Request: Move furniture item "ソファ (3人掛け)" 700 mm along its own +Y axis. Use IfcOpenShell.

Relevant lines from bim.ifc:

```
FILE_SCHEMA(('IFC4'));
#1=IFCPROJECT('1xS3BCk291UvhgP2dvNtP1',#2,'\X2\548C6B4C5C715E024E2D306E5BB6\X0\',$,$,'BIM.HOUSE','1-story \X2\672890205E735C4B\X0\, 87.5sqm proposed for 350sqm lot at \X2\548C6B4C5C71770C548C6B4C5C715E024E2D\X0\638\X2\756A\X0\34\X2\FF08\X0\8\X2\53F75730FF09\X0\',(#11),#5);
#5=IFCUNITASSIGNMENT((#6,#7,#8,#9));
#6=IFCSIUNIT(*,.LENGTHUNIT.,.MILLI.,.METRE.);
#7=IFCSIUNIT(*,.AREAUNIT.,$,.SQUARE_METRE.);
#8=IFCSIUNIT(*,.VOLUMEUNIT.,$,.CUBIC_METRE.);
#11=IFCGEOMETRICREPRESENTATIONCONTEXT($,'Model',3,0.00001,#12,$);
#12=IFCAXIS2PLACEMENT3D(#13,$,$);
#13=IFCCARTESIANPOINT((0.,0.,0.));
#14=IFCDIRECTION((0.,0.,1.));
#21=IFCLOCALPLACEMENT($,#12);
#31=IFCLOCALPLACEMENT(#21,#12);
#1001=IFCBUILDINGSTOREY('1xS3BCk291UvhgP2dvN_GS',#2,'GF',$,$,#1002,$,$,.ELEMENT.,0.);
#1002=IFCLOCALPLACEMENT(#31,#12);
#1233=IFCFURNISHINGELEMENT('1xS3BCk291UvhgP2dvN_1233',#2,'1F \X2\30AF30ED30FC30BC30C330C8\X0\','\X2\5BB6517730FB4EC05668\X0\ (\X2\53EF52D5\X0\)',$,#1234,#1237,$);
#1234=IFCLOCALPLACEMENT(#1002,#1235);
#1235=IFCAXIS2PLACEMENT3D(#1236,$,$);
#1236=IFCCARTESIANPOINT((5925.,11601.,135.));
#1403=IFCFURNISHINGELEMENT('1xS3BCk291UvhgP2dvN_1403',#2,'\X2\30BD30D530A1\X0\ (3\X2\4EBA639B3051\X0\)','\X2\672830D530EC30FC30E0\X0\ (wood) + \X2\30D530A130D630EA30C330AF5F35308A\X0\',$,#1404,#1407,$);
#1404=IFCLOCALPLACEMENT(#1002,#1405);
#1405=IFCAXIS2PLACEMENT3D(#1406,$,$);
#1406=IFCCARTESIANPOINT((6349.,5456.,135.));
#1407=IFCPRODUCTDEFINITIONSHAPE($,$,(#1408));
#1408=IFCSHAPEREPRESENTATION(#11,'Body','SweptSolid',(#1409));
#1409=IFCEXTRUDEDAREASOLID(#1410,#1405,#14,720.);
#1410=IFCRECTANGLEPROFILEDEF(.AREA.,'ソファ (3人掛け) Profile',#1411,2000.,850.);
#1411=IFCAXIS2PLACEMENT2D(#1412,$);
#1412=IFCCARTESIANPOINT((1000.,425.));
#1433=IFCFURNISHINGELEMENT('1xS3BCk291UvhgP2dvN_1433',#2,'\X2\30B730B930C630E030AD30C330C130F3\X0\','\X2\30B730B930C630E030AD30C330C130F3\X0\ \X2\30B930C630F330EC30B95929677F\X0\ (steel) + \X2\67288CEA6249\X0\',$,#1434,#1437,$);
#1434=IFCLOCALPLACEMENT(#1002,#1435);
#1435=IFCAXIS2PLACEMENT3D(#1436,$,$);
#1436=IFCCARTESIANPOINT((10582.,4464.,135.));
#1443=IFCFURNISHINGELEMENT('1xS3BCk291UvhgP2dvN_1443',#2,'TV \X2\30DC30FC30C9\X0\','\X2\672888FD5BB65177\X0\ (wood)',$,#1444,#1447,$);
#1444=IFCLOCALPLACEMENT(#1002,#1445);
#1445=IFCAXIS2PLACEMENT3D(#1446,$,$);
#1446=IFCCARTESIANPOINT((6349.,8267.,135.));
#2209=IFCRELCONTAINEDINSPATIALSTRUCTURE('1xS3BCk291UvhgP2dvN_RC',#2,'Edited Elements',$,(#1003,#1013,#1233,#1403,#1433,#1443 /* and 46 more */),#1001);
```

```python
import ifcopenshell
import ifcopenshell.api.geometry
import ifcopenshell.util.placement

model = ifcopenshell.open("bim.ifc")

item = model.by_guid("1xS3BCk291UvhgP2dvN_1403")
matrix = ifcopenshell.util.placement.get_local_placement(item.ObjectPlacement)
matrix[:3, 3] += matrix[:3, 1] * 700.0
ifcopenshell.api.geometry.edit_object_placement(model, product=item, matrix=matrix, is_si=False)

print(ifcopenshell.util.placement.get_local_placement(item.ObjectPlacement).round(3) + 0.0)

model.write("bim_rev.ifc")
```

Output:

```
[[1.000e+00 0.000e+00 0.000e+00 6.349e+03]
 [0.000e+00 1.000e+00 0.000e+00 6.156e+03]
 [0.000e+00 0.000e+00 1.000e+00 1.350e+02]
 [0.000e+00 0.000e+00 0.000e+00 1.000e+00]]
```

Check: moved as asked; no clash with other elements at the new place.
